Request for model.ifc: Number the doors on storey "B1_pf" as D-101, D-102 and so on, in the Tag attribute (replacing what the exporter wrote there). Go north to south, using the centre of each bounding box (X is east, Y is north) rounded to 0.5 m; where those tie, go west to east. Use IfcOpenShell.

First a look at what the model holds.

```python
import ifcopenshell
import ifcopenshell.util.element
import ifcopenshell.util.placement

model = ifcopenshell.open("model.ifc")
print(model.schema)
storey = next(s for s in model.by_type("IfcBuildingStorey") if s.Name == "B1_pf")
doors = [e for e in ifcopenshell.util.element.get_decomposition(storey) if e.is_a("IfcDoor")]
for e in sorted(doors, key=lambda e: e.id()):
    origin = ifcopenshell.util.placement.get_local_placement(e.ObjectPlacement)[:3, 3]
    print(e.id(), e.Tag, e.Name, origin.round(2) + 0.0, sep=" | ")
```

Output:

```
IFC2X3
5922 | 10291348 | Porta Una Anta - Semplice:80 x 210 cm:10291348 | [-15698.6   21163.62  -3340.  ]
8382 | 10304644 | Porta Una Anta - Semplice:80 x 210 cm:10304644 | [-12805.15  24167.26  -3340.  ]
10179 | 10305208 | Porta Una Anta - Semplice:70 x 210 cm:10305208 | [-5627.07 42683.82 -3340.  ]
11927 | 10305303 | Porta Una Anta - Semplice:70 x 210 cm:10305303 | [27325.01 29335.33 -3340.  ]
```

```python
import ifcopenshell
import ifcopenshell.geom
import ifcopenshell.util.element
import ifcopenshell.util.shape

model = ifcopenshell.open("model.ifc")
settings = ifcopenshell.geom.settings()
settings.set("use-world-coords", True)


def centre(element):
    shape = ifcopenshell.geom.create_shape(settings, element)
    return ifcopenshell.util.shape.get_bbox_centroid(shape.geometry)


storey = next(s for s in model.by_type("IfcBuildingStorey") if s.Name == "B1_pf")
doors = [e for e in ifcopenshell.util.element.get_decomposition(storey) if e.is_a("IfcDoor")]

# Insertion points can sit at a corner or the storey origin, so sort by the geometry (in metres).
centres = {e: centre(e) for e in doors}
doors.sort(key=lambda e: (-round(centres[e][1] / 0.5), centres[e][0]))

for i, e in enumerate(doors, start=1):
    number = f"D-1{i:02d}"
    e.Tag = number
    print(e.id(), number)

model.write("model_rev.ifc")
```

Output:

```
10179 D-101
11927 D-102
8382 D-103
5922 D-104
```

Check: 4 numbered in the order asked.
